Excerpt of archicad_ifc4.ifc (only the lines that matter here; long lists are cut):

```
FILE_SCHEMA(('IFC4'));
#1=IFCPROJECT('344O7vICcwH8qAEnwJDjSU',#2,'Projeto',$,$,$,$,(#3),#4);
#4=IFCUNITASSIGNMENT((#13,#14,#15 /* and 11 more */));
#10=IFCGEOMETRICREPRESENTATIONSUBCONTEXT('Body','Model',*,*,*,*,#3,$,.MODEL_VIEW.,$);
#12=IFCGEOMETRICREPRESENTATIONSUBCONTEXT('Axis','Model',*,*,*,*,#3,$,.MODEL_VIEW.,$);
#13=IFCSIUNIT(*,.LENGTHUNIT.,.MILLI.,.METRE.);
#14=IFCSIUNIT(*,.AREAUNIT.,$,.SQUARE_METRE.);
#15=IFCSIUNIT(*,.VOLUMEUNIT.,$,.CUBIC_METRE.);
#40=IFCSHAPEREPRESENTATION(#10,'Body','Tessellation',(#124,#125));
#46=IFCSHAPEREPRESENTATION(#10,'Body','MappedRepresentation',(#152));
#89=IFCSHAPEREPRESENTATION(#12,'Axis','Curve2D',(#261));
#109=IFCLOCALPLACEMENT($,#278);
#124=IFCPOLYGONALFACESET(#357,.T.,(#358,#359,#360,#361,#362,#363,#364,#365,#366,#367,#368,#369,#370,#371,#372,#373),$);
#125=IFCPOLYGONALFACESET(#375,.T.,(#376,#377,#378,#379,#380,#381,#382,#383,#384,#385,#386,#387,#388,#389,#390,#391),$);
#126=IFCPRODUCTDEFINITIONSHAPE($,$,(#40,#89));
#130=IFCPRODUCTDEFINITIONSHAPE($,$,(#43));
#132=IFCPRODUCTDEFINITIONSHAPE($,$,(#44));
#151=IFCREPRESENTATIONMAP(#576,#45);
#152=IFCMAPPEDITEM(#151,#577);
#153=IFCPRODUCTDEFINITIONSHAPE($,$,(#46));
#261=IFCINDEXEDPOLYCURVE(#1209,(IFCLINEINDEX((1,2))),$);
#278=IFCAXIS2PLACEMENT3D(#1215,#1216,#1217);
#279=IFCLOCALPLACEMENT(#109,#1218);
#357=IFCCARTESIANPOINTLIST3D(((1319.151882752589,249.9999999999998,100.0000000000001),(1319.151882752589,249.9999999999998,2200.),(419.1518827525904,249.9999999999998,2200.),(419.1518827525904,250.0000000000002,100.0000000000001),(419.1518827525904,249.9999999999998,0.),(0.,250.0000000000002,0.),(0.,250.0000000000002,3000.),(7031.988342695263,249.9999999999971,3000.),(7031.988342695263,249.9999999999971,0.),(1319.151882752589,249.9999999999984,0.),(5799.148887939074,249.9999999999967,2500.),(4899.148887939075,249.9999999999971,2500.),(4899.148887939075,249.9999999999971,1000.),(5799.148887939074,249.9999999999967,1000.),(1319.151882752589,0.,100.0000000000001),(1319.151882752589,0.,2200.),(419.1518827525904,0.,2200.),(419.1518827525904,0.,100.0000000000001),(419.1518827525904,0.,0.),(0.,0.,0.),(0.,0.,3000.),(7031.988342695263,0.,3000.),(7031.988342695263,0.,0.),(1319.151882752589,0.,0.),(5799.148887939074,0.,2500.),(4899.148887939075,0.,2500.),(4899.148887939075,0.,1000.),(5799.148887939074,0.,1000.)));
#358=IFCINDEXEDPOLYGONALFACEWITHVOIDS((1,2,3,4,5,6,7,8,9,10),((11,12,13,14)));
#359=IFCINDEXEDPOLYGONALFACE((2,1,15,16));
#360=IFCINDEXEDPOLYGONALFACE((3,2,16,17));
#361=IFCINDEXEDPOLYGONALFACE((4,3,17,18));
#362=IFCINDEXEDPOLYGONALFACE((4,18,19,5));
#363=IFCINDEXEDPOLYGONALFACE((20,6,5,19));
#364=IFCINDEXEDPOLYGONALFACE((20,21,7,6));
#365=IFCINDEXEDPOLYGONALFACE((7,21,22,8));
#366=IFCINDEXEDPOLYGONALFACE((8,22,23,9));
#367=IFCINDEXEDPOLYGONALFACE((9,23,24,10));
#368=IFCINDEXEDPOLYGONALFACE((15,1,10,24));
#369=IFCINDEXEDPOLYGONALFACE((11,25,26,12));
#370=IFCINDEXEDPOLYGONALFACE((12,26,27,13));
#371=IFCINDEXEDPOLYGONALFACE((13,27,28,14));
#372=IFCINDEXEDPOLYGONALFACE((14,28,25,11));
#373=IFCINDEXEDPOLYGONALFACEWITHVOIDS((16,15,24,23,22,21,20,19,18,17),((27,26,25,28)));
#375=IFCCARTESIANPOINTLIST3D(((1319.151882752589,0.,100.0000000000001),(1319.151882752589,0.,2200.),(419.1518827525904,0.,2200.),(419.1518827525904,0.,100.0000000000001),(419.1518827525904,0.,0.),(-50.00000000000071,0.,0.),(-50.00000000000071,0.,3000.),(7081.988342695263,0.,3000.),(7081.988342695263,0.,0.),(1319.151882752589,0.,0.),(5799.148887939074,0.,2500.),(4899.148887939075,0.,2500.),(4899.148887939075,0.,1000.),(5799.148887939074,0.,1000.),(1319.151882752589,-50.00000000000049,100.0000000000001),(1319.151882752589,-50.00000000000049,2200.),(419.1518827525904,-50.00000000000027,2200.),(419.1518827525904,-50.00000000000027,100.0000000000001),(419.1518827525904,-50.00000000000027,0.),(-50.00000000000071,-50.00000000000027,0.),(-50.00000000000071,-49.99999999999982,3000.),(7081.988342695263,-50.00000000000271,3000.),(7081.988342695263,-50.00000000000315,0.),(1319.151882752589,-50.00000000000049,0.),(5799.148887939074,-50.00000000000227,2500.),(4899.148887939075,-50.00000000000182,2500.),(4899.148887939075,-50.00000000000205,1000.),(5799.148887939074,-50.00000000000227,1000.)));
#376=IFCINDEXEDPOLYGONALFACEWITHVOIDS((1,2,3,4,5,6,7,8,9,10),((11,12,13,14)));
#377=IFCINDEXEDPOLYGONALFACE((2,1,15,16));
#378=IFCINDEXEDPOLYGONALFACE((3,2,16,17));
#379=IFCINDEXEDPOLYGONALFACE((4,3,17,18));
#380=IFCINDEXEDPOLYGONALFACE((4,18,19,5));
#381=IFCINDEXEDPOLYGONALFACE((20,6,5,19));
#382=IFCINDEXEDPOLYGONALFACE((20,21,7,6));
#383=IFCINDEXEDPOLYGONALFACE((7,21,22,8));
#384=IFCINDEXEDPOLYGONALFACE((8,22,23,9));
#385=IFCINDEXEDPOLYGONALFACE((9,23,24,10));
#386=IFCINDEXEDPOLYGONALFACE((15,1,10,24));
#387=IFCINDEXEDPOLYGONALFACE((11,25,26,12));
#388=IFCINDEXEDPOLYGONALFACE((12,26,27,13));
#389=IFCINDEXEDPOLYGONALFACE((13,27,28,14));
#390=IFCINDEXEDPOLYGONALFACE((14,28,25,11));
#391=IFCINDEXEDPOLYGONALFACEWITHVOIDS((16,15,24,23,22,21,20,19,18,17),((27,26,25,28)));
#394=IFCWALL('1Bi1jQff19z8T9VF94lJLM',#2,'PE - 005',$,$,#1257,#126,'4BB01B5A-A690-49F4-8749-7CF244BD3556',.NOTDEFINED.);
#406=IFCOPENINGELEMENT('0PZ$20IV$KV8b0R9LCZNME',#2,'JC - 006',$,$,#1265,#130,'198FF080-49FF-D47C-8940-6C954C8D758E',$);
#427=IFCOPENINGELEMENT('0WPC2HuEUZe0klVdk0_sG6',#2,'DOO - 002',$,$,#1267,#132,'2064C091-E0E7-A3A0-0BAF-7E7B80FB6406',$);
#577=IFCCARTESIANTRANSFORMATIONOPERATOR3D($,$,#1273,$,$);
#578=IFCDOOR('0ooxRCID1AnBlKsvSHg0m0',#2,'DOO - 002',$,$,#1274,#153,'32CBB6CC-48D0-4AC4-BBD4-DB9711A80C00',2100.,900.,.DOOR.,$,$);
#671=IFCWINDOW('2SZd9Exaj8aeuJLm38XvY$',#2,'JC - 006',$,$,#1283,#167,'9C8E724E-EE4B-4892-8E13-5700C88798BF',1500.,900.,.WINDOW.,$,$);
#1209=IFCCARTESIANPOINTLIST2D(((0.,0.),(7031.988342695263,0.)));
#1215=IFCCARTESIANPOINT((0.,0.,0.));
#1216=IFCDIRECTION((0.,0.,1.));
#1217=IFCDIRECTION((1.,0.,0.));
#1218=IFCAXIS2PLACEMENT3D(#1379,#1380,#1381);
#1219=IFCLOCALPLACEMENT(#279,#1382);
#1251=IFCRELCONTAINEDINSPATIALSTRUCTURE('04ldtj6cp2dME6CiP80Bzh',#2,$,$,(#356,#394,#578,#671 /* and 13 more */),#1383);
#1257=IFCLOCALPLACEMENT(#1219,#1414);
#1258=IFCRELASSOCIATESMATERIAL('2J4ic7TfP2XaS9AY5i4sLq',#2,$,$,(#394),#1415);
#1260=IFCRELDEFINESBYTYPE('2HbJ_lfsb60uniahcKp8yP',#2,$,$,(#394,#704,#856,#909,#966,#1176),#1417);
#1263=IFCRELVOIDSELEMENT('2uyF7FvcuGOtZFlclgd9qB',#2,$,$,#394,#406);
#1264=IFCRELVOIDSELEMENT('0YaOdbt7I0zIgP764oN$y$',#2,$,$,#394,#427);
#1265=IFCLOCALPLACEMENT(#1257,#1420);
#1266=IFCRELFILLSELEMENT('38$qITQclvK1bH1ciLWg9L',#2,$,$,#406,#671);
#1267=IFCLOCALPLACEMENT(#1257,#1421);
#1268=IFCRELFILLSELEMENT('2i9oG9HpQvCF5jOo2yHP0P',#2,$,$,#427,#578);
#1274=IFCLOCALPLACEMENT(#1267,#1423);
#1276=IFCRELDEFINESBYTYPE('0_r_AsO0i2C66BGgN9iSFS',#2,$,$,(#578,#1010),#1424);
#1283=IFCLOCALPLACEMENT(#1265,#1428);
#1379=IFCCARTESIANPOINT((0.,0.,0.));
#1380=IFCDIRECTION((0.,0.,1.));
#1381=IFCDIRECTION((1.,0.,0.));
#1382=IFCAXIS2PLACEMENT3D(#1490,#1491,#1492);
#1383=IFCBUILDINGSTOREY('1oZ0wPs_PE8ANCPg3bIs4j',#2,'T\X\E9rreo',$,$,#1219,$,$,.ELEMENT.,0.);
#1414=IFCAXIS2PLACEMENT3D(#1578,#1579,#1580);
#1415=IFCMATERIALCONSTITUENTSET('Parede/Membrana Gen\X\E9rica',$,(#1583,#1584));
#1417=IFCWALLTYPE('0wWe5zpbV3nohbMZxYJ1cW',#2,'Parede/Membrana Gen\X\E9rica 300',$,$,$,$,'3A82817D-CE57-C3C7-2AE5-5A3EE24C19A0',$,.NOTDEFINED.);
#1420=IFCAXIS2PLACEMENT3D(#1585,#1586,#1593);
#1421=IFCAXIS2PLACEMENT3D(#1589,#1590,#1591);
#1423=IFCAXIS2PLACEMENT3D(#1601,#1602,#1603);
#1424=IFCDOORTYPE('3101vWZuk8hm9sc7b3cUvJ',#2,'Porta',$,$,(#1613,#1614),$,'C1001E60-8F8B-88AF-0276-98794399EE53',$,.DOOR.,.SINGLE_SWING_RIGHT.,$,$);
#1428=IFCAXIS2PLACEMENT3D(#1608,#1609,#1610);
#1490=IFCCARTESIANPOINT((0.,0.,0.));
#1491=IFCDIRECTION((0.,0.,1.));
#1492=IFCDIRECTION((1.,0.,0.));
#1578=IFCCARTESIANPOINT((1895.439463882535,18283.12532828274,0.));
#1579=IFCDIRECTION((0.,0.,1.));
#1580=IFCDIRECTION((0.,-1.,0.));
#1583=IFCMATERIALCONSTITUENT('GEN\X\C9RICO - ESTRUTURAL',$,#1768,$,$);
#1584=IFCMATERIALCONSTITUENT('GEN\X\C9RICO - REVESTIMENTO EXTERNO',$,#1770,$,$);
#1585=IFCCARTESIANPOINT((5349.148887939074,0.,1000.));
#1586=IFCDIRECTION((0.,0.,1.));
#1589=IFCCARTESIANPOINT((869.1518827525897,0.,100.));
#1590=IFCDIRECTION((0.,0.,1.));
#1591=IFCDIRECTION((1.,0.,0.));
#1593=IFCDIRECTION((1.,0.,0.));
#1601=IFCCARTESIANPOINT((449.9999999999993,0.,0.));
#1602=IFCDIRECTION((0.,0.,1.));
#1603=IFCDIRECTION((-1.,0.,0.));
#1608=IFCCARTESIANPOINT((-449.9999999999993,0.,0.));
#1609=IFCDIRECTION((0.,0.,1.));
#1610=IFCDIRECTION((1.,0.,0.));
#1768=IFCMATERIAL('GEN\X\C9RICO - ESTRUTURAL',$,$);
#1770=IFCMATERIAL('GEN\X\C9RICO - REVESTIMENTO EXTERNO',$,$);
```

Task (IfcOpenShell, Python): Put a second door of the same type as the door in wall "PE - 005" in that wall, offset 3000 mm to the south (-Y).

```python
import ifcopenshell
import ifcopenshell.api.feature
import ifcopenshell.api.geometry
import ifcopenshell.api.root
import ifcopenshell.geom
import ifcopenshell.util.element
import ifcopenshell.util.placement
import ifcopenshell.util.shape

model = ifcopenshell.open("archicad_ifc4.ifc")
settings = ifcopenshell.geom.settings()


def volume(element):
    """Net volume in cubic metres, openings subtracted."""
    shape = ifcopenshell.geom.create_shape(settings, element)
    return ifcopenshell.util.shape.get_volume(shape.geometry)


def reuse_history(source, copy):
    """copy_class also copies each property set's owner history, people and application; keep the originals."""
    for rel in copy.IsDefinedBy:
        if rel.is_a("IfcRelDefinesByProperties") and (history := rel.RelatingPropertyDefinition.OwnerHistory):
            rel.RelatingPropertyDefinition.OwnerHistory = source.OwnerHistory
            ifcopenshell.util.element.remove_deep2(model, history)


door = model.by_guid("0ooxRCID1AnBlKsvSHg0m0")
opening = door.FillsVoids[0].RelatingOpeningElement
wall = opening.VoidsElements[0].RelatingBuildingElement
before = volume(wall)
shift = ifcopenshell.util.placement.get_local_placement(wall.ObjectPlacement)[:3, 0] * 3000.0

# copy_class copies the void relationship, type, container and properties, but no geometry.
new_opening = ifcopenshell.api.root.copy_class(model, product=opening)
new_opening.Representation = ifcopenshell.util.element.copy_deep(
    model, opening.Representation, exclude=["IfcGeometricRepresentationContext", "IfcRepresentationMap"]
)
new_opening.Tag = None
new_door = ifcopenshell.api.root.copy_class(model, product=door)
new_door.Representation = ifcopenshell.util.element.copy_deep(
    model, door.Representation, exclude=["IfcGeometricRepresentationContext", "IfcRepresentationMap"]
)
new_door.Tag = None
reuse_history(door, new_door)
ifcopenshell.api.feature.add_filling(model, opening=new_opening, element=new_door)

for old, new in ((opening, new_opening), (door, new_door)):
    matrix = ifcopenshell.util.placement.get_local_placement(old.ObjectPlacement)
    matrix[:3, 3] += shift
    ifcopenshell.api.geometry.edit_object_placement(model, product=new, matrix=matrix, is_si=False)

after = volume(wall)

print(f"wall volume {before:.3f} -> {after:.3f} m3")

model.write("archicad_ifc4-out.ifc")
```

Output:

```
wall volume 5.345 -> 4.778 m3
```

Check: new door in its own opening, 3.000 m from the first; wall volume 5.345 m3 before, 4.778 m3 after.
